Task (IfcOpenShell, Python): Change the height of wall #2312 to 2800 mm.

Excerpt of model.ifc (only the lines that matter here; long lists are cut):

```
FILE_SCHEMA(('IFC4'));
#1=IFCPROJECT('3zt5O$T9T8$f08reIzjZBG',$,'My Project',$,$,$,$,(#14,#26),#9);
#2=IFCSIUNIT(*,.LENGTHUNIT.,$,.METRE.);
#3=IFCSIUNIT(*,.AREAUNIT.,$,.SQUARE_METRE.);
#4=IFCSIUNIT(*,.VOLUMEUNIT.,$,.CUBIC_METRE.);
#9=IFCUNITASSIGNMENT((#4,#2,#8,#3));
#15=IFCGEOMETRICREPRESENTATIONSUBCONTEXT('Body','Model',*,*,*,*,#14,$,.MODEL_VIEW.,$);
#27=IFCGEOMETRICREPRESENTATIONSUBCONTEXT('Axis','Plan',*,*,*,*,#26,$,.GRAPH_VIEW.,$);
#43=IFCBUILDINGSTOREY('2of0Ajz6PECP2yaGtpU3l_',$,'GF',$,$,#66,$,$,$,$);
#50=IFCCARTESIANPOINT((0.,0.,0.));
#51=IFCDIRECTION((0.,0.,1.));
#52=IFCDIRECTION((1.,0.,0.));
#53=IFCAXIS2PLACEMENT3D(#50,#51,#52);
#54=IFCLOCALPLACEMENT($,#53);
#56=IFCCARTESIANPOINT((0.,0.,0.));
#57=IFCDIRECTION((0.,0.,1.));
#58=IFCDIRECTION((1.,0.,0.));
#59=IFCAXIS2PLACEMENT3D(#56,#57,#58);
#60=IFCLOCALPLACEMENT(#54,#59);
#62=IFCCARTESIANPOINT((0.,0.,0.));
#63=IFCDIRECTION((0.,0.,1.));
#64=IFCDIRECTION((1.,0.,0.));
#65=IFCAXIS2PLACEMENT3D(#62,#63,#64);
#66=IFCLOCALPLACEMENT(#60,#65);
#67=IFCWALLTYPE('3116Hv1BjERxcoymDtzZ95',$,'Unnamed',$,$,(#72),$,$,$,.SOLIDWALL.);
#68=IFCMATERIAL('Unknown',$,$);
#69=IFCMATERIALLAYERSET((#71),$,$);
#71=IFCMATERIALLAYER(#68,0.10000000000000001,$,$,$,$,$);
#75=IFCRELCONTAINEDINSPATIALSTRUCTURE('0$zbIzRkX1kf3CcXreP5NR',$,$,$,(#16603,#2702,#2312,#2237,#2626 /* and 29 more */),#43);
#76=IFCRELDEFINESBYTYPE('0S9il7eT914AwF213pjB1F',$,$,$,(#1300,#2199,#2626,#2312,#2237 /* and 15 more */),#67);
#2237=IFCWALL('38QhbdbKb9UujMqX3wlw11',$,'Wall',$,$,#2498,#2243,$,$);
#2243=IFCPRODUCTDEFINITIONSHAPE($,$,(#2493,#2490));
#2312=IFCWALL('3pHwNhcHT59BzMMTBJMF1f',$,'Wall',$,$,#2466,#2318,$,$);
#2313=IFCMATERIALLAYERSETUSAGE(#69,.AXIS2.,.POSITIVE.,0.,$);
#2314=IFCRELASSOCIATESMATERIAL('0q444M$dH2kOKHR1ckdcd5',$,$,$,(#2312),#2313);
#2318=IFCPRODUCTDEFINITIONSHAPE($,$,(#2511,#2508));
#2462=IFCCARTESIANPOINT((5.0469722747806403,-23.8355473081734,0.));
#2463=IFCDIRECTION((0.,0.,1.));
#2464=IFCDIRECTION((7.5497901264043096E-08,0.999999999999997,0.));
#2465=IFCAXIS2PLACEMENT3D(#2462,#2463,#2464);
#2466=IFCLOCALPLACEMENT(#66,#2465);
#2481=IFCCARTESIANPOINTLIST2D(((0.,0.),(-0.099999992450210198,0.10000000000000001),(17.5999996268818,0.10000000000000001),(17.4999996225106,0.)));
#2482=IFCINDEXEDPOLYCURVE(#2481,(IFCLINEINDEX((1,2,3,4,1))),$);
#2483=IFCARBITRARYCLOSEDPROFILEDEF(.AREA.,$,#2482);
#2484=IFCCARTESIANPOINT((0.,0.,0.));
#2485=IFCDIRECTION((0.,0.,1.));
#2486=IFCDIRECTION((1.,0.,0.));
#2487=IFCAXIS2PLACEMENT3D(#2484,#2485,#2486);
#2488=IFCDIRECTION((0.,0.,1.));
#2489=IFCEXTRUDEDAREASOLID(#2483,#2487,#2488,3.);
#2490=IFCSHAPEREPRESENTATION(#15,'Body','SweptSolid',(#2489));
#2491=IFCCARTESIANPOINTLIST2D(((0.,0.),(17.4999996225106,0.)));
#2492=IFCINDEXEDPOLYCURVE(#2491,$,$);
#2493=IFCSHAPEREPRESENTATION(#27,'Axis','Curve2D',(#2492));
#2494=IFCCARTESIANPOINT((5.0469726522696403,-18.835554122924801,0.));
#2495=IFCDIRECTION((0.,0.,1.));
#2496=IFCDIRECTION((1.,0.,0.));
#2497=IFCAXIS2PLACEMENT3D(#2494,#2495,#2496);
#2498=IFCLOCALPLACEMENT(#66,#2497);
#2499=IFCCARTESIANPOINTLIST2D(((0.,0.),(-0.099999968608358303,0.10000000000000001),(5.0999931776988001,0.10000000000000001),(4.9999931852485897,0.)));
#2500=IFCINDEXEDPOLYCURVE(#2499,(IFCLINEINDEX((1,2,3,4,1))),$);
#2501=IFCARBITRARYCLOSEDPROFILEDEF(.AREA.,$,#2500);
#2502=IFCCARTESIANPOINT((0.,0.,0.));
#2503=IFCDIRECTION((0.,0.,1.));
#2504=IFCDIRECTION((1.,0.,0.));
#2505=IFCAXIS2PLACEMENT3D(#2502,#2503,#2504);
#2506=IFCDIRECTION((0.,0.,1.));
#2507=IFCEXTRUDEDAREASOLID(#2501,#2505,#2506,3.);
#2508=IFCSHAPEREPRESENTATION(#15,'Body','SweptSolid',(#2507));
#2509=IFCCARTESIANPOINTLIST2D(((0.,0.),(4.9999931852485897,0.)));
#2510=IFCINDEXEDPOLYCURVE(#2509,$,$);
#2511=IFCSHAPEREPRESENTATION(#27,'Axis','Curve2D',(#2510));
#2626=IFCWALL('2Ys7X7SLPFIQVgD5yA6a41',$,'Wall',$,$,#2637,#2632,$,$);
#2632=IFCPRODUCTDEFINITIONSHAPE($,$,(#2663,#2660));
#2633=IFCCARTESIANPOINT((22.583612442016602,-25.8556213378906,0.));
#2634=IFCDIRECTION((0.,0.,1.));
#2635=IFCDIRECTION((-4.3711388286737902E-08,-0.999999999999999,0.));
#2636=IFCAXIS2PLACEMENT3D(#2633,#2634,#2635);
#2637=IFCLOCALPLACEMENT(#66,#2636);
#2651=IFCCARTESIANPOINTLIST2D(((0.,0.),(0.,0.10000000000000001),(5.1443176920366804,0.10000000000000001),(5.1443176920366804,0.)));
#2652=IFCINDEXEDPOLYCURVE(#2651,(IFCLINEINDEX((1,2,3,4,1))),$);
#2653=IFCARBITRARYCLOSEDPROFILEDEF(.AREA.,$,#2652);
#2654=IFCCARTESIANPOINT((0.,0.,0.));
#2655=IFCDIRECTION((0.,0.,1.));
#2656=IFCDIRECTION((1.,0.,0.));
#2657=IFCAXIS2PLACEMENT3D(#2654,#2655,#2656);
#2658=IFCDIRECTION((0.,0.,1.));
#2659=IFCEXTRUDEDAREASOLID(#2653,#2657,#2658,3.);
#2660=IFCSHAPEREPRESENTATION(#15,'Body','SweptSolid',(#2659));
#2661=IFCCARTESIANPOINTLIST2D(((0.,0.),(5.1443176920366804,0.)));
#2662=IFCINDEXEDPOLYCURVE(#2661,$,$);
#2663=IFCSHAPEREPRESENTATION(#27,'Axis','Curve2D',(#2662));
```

```python
import ifcopenshell
import ifcopenshell.geom
import ifcopenshell.util.representation
import ifcopenshell.util.shape

model = ifcopenshell.open("model.ifc")
settings = ifcopenshell.geom.settings()


def volume(element):
    """Net volume in cubic metres, openings subtracted."""
    shape = ifcopenshell.geom.create_shape(settings, element)
    return ifcopenshell.util.shape.get_volume(shape.geometry)


wall = model.by_guid("3pHwNhcHT59BzMMTBJMF1f")
before = volume(wall)

body = ifcopenshell.util.representation.get_representation(wall, "Model", "Body")
solid = body.Items[0]
old_height = solid.Depth
solid.Depth = 2.8
after = volume(wall)

print(f"height {old_height:g} -> {solid.Depth:g}, volume {before:.3f} -> {after:.3f} m3")

model.write("model_updated.ifc")
```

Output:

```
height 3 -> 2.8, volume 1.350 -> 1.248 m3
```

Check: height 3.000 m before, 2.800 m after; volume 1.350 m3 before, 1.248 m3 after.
